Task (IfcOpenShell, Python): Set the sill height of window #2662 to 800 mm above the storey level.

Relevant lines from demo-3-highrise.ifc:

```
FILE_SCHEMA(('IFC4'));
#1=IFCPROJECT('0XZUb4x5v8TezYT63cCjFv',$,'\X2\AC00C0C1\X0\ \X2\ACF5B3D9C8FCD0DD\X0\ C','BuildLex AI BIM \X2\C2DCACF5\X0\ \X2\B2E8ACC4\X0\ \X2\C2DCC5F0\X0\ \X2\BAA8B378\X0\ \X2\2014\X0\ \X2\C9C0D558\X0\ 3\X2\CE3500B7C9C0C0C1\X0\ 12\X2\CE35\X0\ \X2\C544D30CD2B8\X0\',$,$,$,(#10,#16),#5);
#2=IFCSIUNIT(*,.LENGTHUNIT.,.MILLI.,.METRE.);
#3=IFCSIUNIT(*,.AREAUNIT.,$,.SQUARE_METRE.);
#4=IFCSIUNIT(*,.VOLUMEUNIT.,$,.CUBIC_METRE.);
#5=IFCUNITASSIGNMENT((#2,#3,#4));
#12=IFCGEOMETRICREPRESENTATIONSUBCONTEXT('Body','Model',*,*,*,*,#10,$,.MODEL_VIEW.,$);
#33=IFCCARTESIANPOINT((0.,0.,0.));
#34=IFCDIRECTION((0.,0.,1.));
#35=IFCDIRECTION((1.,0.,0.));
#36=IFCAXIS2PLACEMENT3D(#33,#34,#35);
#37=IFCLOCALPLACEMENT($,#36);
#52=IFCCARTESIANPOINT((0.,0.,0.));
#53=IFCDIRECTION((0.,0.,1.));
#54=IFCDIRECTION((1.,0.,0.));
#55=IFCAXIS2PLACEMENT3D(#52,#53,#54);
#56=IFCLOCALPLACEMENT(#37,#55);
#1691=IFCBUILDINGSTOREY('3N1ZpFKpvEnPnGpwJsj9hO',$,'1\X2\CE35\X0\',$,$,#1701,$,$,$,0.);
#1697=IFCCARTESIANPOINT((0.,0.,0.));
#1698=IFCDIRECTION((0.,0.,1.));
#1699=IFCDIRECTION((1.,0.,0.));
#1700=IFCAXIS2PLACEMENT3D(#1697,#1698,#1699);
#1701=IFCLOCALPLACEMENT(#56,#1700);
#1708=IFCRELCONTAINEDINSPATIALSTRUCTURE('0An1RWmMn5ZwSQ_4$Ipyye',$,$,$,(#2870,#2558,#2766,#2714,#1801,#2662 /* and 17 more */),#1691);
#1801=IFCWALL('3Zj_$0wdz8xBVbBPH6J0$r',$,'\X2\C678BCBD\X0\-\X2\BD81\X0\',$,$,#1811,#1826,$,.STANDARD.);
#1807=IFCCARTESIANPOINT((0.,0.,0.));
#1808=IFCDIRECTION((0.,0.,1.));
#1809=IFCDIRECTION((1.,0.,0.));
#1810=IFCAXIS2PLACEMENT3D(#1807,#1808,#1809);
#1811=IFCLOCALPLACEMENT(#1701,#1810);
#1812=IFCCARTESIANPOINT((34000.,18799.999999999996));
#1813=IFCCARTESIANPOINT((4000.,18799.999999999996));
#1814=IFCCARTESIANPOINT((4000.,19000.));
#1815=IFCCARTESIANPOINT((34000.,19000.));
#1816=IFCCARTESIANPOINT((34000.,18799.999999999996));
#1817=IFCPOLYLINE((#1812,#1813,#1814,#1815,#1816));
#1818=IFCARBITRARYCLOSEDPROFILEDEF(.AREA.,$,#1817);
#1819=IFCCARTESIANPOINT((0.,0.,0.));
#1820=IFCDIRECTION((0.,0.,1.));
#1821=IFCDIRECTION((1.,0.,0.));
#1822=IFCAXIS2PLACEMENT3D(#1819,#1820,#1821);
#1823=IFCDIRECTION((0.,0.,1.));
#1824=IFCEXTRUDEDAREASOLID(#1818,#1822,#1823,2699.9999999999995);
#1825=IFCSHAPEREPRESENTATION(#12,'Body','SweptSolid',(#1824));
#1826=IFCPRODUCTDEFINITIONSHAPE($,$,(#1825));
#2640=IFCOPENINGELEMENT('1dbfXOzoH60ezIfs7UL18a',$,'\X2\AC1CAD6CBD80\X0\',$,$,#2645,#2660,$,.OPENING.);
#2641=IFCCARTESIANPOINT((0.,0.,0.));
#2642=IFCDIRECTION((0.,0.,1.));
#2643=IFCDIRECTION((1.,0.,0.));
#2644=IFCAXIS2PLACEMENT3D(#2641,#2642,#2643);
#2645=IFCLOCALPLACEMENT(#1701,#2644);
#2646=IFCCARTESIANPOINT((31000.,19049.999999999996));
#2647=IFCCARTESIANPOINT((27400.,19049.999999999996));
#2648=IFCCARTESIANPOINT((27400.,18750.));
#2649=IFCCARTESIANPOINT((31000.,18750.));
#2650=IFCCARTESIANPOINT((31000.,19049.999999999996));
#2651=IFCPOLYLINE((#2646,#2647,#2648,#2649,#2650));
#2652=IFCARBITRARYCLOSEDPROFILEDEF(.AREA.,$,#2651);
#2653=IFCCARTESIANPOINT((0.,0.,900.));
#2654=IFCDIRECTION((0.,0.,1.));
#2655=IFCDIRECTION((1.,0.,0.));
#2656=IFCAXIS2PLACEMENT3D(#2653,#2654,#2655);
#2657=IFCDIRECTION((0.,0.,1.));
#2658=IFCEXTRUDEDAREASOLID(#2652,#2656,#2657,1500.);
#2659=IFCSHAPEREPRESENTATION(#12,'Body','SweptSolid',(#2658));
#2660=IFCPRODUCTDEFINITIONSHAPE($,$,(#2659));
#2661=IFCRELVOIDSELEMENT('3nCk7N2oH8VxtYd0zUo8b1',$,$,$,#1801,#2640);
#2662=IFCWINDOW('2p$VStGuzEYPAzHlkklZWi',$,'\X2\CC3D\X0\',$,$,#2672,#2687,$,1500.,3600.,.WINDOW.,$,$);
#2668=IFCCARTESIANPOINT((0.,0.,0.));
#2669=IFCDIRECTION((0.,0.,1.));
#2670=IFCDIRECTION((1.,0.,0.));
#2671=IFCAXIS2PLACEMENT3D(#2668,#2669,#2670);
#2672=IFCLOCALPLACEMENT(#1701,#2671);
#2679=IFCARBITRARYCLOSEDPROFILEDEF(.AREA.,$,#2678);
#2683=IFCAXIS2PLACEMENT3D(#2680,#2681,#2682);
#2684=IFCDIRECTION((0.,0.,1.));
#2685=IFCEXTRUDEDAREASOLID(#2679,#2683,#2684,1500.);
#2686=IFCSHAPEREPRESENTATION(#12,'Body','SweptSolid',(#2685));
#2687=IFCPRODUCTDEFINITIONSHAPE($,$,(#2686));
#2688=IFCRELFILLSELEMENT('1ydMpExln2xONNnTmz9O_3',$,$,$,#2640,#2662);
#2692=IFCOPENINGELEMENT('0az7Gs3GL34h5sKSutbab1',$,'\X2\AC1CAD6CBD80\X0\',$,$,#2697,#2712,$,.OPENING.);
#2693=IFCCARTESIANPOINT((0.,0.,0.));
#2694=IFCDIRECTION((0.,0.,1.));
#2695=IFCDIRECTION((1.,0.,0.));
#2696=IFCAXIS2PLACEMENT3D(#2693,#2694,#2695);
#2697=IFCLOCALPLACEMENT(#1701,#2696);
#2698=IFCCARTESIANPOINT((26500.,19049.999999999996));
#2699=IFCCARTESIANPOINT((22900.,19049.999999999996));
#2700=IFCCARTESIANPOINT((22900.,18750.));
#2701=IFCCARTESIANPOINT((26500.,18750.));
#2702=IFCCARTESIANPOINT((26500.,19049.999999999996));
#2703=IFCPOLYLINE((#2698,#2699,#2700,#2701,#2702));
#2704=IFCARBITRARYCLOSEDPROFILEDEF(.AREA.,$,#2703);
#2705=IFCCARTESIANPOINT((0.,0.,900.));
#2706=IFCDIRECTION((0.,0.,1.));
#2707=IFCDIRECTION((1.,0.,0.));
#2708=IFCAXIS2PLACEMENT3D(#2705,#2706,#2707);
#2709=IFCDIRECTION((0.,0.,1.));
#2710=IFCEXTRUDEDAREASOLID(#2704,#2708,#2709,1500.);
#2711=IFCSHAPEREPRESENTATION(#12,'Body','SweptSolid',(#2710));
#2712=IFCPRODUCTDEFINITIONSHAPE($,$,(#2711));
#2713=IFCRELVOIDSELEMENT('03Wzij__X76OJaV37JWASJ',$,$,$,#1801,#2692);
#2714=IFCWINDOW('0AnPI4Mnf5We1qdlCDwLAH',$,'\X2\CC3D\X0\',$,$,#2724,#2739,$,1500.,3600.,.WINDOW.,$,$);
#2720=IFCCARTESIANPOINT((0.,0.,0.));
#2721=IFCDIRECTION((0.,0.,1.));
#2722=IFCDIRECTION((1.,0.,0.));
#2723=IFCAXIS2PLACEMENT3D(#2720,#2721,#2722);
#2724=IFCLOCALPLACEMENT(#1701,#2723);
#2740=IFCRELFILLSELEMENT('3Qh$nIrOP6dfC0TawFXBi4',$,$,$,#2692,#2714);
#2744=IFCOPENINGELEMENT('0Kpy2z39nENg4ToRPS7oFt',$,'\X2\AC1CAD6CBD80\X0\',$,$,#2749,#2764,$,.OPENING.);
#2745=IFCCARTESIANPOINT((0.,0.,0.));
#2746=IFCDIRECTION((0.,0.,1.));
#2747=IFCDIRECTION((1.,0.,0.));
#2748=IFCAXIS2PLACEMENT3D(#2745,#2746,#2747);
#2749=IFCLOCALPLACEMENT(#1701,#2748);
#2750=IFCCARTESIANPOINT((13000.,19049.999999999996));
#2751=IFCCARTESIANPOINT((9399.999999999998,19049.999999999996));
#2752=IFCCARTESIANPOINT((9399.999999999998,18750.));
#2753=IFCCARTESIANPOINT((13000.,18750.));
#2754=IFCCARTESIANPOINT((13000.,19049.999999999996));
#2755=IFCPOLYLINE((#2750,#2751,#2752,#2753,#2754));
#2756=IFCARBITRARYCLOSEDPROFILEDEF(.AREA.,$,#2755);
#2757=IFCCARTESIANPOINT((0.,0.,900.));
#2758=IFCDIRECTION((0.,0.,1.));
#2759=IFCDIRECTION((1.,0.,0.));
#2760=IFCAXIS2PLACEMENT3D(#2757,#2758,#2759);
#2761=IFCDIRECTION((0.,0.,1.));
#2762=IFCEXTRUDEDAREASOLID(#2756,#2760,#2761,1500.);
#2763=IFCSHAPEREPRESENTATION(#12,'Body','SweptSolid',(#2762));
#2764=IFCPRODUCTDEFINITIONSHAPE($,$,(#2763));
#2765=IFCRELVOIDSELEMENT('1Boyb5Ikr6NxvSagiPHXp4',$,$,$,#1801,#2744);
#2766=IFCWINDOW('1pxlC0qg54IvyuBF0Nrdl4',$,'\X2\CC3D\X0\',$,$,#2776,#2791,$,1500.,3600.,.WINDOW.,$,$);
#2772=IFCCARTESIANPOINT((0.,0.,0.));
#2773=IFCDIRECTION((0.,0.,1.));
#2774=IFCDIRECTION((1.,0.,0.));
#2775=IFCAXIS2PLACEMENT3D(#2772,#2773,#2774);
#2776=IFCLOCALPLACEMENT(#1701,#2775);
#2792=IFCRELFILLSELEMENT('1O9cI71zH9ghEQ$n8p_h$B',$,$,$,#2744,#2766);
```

```python
import numpy as np
import ifcopenshell
import ifcopenshell.api.geometry
import ifcopenshell.geom
import ifcopenshell.util.element
import ifcopenshell.util.placement
import ifcopenshell.util.shape
import ifcopenshell.util.unit

model = ifcopenshell.open("demo-3-highrise.ifc")
unit_scale = ifcopenshell.util.unit.calculate_unit_scale(model)

window = model.by_id(2662)
opening = window.FillsVoids[0].RelatingOpeningElement
storey = ifcopenshell.util.element.get_container(window, ifc_class="IfcBuildingStorey")
level = ifcopenshell.util.placement.get_local_placement(storey.ObjectPlacement)[2, 3]

# The opening's origin need not be at the sill, so measure its lowest point.
shape = ifcopenshell.geom.create_shape(ifcopenshell.geom.settings(), opening)
bottom = ifcopenshell.util.shape.get_shape_bottom_elevation(shape, shape.geometry) / unit_scale
dz = level + 0.8 / unit_scale - bottom

shift = np.array([0.0, 0.0, dz])
# The window is not placed relative to its opening, so move both.
for product in (opening, window):
    matrix = ifcopenshell.util.placement.get_local_placement(product.ObjectPlacement)
    matrix[:3, 3] += shift
    ifcopenshell.api.geometry.edit_object_placement(model, product=product, matrix=matrix, is_si=False)

print(f"moved by {dz * unit_scale:+.3f} m")

model.write("demo-3-highrise-out.ifc")
```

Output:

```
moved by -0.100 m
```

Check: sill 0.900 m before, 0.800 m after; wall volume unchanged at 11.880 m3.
